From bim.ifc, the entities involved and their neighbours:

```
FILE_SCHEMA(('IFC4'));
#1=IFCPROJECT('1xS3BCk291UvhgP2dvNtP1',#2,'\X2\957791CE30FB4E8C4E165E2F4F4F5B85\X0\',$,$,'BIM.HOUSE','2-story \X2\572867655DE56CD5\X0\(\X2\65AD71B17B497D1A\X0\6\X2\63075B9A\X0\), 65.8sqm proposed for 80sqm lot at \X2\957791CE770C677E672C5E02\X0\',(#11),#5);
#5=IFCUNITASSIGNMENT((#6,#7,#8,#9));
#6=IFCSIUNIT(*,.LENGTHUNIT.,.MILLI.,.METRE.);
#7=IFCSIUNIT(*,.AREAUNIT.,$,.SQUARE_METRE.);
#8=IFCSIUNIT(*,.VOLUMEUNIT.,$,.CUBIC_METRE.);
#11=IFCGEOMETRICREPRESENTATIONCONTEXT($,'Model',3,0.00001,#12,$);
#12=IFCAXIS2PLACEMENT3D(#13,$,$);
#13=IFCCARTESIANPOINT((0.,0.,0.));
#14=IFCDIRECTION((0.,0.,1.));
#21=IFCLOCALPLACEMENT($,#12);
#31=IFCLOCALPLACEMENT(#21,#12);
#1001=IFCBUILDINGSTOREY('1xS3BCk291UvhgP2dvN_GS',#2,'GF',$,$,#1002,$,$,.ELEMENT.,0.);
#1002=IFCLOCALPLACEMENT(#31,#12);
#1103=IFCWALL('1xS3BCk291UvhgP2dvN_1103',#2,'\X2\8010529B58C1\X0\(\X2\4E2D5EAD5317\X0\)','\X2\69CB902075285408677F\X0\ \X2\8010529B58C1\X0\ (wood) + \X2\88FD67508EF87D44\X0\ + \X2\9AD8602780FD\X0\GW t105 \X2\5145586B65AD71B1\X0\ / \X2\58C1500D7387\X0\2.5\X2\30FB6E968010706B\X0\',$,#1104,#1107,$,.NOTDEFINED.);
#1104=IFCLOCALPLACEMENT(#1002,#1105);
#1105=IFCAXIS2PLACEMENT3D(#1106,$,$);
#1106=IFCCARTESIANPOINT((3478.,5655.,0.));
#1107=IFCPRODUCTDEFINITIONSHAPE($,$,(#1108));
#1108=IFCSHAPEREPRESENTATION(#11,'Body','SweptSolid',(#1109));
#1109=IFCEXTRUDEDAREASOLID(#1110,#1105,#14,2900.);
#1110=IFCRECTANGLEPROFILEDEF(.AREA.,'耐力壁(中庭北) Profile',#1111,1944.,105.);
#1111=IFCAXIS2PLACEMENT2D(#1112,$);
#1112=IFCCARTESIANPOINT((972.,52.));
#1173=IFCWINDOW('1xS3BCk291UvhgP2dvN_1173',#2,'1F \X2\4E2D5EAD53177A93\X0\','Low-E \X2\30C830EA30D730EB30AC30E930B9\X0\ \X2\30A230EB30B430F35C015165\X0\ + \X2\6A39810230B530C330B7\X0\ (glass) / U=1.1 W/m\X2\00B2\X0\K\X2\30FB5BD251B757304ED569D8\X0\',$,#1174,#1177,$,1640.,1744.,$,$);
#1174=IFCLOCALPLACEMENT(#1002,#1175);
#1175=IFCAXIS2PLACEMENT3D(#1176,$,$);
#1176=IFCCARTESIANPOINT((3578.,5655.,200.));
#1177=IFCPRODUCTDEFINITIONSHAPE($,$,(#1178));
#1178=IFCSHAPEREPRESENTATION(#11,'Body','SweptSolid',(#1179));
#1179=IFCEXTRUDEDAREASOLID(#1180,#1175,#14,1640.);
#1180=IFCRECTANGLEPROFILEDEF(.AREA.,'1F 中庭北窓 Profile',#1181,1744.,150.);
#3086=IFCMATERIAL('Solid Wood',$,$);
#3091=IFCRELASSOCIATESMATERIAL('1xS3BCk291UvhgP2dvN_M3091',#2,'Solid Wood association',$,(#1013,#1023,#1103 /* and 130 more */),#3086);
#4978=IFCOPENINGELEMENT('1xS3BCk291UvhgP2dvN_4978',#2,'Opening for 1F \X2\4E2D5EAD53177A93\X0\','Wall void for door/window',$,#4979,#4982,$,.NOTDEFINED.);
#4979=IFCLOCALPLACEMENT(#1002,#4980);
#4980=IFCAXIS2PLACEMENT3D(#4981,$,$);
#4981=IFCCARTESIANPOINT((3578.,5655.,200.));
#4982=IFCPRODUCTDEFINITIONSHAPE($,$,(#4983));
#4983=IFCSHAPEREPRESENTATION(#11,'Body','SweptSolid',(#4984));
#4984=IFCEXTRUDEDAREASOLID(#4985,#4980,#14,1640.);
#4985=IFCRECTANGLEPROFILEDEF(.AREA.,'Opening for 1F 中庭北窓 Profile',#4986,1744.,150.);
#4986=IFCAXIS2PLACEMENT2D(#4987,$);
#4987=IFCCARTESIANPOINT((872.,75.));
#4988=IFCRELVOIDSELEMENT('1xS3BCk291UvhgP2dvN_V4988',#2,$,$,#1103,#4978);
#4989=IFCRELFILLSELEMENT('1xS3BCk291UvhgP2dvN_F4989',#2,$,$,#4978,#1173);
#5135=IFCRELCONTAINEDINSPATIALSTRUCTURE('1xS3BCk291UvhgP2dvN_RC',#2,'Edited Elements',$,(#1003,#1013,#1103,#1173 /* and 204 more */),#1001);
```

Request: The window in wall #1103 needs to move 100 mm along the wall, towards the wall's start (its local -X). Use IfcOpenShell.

```python
import ifcopenshell
import ifcopenshell.api.geometry
import ifcopenshell.util.placement

model = ifcopenshell.open("bim.ifc")

window = model.by_guid("1xS3BCk291UvhgP2dvN_1173")
opening = window.FillsVoids[0].RelatingOpeningElement
wall = opening.VoidsElements[0].RelatingBuildingElement

wall_matrix = ifcopenshell.util.placement.get_local_placement(wall.ObjectPlacement)
shift = wall_matrix[:3, 0] * -100.0
before = ifcopenshell.util.placement.get_local_placement(window.ObjectPlacement)[:3, 3].copy()

# The window is not placed relative to its opening, so move both.
for product in (opening, window):
    matrix = ifcopenshell.util.placement.get_local_placement(product.ObjectPlacement)
    matrix[:3, 3] += shift
    ifcopenshell.api.geometry.edit_object_placement(model, product=product, matrix=matrix, is_si=False)

after = ifcopenshell.util.placement.get_local_placement(window.ObjectPlacement)[:3, 3]
print("window moved by", (after - before).round(3) + 0.0)

model.write("bim_rev.ifc")
```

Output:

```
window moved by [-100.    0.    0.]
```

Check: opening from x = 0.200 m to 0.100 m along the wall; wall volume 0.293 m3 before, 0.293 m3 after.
